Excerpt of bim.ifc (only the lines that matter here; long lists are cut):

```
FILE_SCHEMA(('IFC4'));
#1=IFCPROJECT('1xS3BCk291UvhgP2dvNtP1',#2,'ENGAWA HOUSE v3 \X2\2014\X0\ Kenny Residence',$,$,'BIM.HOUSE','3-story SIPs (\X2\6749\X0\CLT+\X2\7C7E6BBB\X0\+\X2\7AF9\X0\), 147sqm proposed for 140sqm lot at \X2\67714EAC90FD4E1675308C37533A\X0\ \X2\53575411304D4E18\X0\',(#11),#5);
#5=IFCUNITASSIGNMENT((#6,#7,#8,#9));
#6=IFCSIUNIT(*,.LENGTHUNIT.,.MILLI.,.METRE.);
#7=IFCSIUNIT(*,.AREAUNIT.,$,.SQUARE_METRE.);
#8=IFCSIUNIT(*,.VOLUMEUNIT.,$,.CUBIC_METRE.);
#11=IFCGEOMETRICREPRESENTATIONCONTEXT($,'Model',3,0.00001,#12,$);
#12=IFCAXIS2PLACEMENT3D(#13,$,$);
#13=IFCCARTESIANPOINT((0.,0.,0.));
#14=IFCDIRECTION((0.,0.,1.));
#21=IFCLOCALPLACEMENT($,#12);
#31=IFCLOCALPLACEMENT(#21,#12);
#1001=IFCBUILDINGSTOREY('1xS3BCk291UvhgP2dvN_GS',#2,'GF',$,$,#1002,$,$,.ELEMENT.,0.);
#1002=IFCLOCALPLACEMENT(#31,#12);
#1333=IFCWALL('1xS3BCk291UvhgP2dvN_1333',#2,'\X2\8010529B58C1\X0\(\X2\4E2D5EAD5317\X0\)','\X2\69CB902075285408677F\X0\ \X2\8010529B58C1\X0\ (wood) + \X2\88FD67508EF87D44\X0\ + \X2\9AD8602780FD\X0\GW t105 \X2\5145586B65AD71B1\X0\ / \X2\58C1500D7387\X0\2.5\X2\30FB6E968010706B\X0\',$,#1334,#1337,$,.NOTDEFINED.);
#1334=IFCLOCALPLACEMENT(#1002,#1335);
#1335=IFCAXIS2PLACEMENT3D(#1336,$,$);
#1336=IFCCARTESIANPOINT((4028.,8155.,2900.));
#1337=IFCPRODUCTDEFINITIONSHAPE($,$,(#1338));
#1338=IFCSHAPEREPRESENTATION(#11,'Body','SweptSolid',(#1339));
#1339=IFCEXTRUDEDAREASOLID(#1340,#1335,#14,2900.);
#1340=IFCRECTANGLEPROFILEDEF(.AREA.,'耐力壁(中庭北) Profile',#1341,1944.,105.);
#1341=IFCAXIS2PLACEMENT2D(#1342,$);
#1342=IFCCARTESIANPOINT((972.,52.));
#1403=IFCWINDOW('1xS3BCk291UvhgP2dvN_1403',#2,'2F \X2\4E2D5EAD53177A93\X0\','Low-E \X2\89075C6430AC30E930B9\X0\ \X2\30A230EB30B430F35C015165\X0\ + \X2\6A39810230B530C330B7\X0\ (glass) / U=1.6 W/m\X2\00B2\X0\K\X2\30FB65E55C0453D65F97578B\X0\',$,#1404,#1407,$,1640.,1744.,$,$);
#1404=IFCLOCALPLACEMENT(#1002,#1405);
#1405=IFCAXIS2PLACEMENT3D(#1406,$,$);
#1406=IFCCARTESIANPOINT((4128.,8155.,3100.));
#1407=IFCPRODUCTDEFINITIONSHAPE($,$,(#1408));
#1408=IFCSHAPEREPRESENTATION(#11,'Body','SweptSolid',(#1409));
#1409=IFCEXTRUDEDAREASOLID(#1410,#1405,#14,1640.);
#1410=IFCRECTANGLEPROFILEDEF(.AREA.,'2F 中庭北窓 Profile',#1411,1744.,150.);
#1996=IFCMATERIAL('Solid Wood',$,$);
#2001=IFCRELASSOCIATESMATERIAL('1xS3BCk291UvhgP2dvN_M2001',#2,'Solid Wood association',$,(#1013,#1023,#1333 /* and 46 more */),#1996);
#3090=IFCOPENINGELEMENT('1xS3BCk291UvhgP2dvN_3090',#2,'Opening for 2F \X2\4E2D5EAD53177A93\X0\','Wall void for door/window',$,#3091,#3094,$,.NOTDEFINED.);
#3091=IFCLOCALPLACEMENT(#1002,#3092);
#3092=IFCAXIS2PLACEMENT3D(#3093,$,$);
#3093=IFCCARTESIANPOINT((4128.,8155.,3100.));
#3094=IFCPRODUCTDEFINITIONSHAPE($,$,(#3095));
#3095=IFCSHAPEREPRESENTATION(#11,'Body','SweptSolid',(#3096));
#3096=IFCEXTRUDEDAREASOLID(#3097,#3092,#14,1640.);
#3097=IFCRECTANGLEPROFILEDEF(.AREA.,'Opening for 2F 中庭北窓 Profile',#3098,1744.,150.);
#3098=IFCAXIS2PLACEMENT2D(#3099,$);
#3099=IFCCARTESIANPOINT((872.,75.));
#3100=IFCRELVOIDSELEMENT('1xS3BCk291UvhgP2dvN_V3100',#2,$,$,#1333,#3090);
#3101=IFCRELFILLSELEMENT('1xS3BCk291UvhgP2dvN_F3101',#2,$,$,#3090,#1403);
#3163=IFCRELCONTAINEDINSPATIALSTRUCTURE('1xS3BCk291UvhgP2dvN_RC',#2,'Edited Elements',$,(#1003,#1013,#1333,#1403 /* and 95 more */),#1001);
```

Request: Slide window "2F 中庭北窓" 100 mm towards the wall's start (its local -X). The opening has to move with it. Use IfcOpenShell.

```python
import ifcopenshell
import ifcopenshell.api.geometry
import ifcopenshell.util.placement

model = ifcopenshell.open("bim.ifc")

window = model.by_guid("1xS3BCk291UvhgP2dvN_1403")
opening = window.FillsVoids[0].RelatingOpeningElement
wall = opening.VoidsElements[0].RelatingBuildingElement

wall_matrix = ifcopenshell.util.placement.get_local_placement(wall.ObjectPlacement)
shift = wall_matrix[:3, 0] * -100.0
before = ifcopenshell.util.placement.get_local_placement(window.ObjectPlacement)[:3, 3].copy()

# The window is not placed relative to its opening, so move both.
for product in (opening, window):
    matrix = ifcopenshell.util.placement.get_local_placement(product.ObjectPlacement)
    matrix[:3, 3] += shift
    ifcopenshell.api.geometry.edit_object_placement(model, product=product, matrix=matrix, is_si=False)

after = ifcopenshell.util.placement.get_local_placement(window.ObjectPlacement)[:3, 3]
print("window moved by", (after - before).round(3) + 0.0)

model.write("bim_edited.ifc")
```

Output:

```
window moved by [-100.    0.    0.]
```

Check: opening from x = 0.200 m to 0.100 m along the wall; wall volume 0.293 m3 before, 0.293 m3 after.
